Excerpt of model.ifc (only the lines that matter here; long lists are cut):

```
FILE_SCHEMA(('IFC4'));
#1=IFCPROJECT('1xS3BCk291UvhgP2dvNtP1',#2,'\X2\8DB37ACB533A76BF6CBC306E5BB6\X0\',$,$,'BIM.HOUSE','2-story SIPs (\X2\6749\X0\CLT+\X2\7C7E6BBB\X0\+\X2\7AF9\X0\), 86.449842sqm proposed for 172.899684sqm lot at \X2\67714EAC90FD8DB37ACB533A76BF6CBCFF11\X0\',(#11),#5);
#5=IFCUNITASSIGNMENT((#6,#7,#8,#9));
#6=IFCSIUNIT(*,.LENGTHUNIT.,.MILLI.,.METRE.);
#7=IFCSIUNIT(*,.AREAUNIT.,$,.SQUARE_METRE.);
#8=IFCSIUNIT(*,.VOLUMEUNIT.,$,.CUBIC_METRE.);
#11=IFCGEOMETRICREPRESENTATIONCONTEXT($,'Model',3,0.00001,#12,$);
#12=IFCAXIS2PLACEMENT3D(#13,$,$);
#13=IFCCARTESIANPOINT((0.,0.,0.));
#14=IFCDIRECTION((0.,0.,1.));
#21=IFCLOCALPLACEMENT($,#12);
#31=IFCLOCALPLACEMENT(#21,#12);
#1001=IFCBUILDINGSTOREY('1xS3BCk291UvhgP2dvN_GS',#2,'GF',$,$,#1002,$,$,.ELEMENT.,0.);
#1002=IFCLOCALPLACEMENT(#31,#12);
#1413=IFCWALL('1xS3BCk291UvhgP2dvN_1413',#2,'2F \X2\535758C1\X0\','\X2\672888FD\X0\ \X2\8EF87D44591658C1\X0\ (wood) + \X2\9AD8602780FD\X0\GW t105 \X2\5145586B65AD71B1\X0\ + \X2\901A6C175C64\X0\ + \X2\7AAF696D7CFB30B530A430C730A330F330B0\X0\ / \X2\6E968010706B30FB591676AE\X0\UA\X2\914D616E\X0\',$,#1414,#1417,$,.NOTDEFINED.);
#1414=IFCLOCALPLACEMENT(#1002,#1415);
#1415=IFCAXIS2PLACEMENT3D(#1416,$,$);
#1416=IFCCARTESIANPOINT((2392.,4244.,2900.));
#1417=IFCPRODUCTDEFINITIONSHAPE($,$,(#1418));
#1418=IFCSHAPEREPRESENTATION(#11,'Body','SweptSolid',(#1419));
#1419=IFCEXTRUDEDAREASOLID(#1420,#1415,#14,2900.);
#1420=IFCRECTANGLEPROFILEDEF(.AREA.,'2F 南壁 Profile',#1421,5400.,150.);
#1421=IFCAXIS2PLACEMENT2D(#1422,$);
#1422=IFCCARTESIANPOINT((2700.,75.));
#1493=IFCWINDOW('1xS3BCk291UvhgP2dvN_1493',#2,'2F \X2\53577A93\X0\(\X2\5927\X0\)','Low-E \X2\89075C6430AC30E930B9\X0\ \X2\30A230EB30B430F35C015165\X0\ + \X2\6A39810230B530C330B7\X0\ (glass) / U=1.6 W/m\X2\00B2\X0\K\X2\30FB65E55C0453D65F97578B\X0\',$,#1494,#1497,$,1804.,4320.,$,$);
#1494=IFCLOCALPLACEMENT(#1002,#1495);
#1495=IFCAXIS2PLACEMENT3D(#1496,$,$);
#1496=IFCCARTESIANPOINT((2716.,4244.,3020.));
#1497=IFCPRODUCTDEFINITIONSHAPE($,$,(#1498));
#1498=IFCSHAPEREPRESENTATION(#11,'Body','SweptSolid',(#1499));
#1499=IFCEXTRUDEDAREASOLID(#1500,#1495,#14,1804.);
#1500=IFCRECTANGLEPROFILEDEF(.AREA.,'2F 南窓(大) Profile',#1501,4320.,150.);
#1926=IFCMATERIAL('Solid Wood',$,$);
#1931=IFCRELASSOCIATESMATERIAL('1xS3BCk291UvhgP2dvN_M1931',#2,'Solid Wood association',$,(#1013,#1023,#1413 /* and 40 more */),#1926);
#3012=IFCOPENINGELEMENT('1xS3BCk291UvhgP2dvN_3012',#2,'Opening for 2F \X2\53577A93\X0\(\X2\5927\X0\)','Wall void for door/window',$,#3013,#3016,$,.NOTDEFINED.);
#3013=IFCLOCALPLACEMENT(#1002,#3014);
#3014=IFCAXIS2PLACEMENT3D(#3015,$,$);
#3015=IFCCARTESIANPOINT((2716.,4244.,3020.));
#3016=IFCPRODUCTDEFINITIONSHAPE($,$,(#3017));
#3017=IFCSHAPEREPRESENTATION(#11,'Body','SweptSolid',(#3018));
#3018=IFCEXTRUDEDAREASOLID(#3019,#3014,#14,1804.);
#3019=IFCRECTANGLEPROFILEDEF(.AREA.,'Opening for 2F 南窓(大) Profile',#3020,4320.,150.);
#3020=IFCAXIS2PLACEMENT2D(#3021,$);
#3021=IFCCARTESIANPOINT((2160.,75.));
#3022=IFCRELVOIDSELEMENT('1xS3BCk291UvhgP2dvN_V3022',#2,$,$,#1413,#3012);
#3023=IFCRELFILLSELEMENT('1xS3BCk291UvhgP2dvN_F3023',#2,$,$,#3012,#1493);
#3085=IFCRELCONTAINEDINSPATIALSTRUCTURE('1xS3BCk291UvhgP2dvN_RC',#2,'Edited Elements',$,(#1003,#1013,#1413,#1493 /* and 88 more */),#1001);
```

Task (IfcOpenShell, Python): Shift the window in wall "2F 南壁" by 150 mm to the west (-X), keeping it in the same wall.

```python
import ifcopenshell
import ifcopenshell.api.geometry
import ifcopenshell.util.placement

model = ifcopenshell.open("model.ifc")

window = model.by_guid("1xS3BCk291UvhgP2dvN_1493")
opening = window.FillsVoids[0].RelatingOpeningElement
wall = opening.VoidsElements[0].RelatingBuildingElement

wall_matrix = ifcopenshell.util.placement.get_local_placement(wall.ObjectPlacement)
shift = wall_matrix[:3, 0] * -150.0
before = ifcopenshell.util.placement.get_local_placement(window.ObjectPlacement)[:3, 3].copy()

# The window is not placed relative to its opening, so move both.
for product in (opening, window):
    matrix = ifcopenshell.util.placement.get_local_placement(product.ObjectPlacement)
    matrix[:3, 3] += shift
    ifcopenshell.api.geometry.edit_object_placement(model, product=product, matrix=matrix, is_si=False)

after = ifcopenshell.util.placement.get_local_placement(window.ObjectPlacement)[:3, 3]
print("window moved by", (after - before).round(3) + 0.0)

model.write("model_rev.ifc")
```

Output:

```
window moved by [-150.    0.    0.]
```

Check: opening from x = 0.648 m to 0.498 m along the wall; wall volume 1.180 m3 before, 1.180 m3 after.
